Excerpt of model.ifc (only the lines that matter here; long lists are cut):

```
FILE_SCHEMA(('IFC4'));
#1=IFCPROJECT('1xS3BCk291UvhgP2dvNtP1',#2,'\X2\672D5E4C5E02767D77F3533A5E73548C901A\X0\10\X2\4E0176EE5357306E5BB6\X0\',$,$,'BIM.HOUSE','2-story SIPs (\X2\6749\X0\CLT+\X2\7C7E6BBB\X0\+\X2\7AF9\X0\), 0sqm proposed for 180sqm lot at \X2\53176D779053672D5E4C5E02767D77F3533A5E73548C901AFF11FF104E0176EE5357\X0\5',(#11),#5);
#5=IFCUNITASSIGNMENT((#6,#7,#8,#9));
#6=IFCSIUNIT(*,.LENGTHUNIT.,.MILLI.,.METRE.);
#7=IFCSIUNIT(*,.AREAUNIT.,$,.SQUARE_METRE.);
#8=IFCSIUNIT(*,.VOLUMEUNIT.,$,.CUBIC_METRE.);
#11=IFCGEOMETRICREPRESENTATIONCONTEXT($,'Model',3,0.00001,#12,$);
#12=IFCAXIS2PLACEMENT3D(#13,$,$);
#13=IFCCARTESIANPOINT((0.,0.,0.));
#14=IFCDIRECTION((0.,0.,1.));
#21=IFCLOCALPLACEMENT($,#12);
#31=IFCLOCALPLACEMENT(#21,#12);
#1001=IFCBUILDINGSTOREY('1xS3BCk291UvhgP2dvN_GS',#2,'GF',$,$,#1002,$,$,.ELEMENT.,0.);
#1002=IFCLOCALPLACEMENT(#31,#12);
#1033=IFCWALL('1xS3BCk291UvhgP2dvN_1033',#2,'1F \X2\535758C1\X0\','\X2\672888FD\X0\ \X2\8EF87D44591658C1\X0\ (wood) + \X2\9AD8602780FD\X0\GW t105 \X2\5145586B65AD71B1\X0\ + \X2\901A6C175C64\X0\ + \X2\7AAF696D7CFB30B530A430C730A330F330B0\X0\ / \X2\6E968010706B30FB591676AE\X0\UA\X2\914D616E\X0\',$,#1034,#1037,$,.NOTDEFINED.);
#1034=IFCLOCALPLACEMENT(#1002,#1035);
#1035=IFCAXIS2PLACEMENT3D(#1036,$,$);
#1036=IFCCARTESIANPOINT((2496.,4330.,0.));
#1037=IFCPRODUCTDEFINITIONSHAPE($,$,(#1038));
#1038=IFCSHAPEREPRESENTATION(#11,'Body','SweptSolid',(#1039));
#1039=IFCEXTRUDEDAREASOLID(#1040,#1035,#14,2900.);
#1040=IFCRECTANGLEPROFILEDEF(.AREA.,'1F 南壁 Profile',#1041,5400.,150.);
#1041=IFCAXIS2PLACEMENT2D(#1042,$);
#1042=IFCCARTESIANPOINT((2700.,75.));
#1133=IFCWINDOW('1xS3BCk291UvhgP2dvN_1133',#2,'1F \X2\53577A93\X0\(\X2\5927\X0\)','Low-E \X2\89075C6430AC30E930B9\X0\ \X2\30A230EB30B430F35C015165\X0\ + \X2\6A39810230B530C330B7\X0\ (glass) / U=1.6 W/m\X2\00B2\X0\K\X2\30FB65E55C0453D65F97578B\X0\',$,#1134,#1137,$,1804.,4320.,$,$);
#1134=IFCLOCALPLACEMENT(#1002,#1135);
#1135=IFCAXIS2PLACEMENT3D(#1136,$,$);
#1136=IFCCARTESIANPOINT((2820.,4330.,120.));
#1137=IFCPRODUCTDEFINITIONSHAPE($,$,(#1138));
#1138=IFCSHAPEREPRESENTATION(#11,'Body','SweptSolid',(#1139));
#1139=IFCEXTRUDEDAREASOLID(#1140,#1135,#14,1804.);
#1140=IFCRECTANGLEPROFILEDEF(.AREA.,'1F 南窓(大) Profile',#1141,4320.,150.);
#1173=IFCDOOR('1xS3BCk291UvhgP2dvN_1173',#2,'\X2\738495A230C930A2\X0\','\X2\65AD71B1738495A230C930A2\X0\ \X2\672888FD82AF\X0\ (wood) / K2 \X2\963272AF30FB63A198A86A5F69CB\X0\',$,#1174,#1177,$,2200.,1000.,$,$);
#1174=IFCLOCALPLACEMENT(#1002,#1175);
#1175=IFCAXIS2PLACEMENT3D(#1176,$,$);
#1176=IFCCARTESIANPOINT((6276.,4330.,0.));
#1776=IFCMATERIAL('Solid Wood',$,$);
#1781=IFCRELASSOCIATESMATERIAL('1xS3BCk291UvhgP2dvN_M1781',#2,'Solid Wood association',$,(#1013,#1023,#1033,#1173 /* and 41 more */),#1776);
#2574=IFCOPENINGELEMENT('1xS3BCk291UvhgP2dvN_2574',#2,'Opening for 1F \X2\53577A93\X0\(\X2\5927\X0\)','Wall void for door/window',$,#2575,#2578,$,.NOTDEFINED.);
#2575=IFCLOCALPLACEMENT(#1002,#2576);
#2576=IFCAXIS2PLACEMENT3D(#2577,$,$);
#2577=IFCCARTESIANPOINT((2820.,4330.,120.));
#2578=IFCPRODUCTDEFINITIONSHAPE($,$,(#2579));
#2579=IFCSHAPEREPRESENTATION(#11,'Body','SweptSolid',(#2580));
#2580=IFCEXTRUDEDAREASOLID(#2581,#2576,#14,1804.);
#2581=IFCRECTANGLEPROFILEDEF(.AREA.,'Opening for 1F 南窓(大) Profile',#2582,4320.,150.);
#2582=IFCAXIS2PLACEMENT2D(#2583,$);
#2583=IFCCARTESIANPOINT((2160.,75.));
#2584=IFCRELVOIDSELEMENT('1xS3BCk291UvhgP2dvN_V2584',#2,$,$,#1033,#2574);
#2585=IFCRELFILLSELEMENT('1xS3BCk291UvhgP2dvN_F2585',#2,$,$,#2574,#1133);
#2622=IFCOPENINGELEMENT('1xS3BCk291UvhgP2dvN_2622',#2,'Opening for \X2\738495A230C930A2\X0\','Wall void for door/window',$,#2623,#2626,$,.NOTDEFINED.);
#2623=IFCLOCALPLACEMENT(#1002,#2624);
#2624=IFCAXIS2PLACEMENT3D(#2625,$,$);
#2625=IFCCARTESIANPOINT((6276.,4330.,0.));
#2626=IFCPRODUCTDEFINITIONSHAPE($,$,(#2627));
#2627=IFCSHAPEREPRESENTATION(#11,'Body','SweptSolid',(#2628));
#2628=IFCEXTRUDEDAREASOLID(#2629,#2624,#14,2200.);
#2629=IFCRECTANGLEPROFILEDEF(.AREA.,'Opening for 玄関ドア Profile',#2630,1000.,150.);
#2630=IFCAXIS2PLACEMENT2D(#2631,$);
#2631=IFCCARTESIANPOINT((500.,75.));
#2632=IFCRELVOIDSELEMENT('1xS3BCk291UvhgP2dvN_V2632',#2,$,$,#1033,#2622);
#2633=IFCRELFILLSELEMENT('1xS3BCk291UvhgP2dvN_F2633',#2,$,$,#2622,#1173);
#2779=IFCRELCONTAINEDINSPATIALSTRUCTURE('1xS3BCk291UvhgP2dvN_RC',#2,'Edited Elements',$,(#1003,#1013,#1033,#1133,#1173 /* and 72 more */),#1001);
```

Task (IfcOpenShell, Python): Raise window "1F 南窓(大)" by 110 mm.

```python
import numpy as np
import ifcopenshell
import ifcopenshell.api.geometry
import ifcopenshell.util.placement
import ifcopenshell.util.unit

model = ifcopenshell.open("model.ifc")
unit_scale = ifcopenshell.util.unit.calculate_unit_scale(model)

window = model.by_guid("1xS3BCk291UvhgP2dvN_1133")
opening = window.FillsVoids[0].RelatingOpeningElement
dz = 110.0

shift = np.array([0.0, 0.0, dz])
# The window is not placed relative to its opening, so move both.
for product in (opening, window):
    matrix = ifcopenshell.util.placement.get_local_placement(product.ObjectPlacement)
    matrix[:3, 3] += shift
    ifcopenshell.api.geometry.edit_object_placement(model, product=product, matrix=matrix, is_si=False)

print(f"moved by {dz * unit_scale:+.3f} m")

model.write("model-out.ifc")
```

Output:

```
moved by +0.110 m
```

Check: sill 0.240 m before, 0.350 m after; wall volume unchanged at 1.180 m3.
